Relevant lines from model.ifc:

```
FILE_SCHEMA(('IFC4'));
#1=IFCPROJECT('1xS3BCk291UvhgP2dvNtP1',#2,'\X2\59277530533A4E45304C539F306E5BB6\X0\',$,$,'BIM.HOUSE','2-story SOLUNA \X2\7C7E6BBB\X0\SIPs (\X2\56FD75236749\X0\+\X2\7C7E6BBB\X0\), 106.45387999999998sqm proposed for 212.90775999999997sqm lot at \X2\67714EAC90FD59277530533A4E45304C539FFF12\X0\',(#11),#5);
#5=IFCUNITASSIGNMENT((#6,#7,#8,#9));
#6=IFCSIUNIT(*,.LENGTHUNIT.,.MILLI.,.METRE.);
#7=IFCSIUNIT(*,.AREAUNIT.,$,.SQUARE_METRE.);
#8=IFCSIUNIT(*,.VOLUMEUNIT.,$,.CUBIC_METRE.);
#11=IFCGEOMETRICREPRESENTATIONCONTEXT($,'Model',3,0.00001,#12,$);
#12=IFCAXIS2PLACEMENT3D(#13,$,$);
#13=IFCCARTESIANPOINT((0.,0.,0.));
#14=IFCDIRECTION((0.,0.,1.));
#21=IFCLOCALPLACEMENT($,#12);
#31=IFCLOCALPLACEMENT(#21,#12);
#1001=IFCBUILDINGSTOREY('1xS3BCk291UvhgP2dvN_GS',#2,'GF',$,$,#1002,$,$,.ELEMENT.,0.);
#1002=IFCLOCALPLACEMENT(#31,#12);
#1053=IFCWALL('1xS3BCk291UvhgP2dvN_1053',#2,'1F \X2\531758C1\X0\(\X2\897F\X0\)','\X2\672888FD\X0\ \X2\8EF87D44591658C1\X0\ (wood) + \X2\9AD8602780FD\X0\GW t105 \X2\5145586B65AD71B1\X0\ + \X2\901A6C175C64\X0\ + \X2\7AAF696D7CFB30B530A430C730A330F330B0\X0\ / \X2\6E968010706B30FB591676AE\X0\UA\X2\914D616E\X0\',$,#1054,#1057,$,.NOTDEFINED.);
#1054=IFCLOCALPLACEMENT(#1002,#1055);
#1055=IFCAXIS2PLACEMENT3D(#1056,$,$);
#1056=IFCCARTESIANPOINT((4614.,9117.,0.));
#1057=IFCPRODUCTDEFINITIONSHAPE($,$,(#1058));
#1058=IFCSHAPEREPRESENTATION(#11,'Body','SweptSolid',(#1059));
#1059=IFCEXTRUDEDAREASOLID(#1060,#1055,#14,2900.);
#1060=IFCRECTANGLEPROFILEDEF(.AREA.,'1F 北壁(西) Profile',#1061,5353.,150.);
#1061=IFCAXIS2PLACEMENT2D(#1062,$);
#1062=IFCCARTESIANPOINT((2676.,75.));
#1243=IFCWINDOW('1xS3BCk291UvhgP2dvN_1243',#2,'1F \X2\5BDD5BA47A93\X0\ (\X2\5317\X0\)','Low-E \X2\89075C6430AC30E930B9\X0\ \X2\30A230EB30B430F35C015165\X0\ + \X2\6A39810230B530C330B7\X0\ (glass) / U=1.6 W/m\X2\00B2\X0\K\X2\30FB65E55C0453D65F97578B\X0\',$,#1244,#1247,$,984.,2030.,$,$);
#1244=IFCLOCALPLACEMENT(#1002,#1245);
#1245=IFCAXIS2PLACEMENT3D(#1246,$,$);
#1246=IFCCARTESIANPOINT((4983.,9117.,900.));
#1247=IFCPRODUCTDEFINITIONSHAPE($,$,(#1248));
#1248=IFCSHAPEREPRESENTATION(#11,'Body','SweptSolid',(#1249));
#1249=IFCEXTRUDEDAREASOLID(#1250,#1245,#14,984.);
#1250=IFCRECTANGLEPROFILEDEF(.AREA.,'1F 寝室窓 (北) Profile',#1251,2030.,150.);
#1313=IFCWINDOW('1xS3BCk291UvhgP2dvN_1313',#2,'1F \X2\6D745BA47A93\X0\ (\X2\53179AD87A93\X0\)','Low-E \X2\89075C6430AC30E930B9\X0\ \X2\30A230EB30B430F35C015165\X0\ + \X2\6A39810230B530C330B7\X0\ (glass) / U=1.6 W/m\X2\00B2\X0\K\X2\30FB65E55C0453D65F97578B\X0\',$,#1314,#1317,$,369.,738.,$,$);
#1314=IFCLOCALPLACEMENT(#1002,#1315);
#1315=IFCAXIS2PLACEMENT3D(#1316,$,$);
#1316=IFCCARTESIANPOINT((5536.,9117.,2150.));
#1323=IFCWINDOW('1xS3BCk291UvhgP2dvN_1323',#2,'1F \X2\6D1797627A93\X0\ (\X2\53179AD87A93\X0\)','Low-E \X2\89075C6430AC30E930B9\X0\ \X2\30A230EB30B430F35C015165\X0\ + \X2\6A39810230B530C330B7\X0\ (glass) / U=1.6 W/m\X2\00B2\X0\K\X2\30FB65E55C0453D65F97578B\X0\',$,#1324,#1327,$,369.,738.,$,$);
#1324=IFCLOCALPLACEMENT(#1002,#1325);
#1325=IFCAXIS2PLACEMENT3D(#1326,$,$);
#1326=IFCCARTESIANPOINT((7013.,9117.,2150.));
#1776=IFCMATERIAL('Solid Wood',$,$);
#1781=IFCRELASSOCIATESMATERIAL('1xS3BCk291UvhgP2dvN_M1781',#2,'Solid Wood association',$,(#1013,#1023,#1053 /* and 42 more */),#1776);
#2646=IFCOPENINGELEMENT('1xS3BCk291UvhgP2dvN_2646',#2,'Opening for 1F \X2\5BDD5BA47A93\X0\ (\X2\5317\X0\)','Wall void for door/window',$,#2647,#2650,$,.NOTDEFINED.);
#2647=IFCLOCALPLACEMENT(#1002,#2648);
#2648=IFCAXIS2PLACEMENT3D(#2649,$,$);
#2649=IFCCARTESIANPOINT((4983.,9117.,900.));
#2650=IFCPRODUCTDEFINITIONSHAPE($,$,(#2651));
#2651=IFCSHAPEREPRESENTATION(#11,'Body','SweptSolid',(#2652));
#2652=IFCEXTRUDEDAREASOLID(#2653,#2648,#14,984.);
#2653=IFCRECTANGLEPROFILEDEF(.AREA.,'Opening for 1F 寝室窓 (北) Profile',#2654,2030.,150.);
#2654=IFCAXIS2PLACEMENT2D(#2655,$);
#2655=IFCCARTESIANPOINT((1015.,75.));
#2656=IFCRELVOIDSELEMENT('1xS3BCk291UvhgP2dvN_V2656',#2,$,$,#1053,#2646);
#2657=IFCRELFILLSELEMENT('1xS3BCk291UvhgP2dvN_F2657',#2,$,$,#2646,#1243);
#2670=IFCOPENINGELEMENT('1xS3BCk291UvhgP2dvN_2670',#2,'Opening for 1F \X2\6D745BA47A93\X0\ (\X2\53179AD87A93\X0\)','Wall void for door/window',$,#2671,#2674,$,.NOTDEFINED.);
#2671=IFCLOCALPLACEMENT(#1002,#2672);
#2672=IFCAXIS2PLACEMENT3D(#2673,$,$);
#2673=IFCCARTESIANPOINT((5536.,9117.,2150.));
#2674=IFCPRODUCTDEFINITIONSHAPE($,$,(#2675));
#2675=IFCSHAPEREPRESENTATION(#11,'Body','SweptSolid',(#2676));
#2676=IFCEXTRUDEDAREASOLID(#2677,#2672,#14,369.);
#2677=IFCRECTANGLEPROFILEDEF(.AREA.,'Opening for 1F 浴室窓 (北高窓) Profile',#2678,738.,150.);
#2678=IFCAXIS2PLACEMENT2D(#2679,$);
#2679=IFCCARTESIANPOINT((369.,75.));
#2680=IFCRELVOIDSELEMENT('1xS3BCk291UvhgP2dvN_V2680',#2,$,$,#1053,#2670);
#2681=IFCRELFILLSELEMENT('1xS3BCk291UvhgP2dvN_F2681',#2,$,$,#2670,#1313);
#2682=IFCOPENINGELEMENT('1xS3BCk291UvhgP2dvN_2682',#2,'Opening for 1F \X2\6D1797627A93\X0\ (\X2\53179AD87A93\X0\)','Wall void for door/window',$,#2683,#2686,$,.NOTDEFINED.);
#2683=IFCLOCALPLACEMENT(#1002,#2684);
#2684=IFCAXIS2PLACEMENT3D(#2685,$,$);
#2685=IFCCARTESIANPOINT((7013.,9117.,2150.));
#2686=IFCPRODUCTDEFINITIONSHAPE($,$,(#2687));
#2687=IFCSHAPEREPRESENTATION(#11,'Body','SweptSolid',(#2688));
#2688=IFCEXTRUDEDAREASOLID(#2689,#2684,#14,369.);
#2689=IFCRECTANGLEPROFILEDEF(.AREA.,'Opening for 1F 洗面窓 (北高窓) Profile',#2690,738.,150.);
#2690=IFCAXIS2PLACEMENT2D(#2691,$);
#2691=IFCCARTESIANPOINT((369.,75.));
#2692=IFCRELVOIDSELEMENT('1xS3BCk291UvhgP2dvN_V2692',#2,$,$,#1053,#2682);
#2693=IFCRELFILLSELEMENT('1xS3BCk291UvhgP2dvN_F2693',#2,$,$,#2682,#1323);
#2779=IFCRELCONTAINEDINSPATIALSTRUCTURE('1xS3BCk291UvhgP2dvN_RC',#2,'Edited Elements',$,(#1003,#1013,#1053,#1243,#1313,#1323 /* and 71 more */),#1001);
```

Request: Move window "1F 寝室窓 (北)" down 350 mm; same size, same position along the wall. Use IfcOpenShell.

```python
import numpy as np
import ifcopenshell
import ifcopenshell.api.geometry
import ifcopenshell.util.placement
import ifcopenshell.util.unit

model = ifcopenshell.open("model.ifc")
unit_scale = ifcopenshell.util.unit.calculate_unit_scale(model)

window = model.by_guid("1xS3BCk291UvhgP2dvN_1243")
opening = window.FillsVoids[0].RelatingOpeningElement
dz = -0.35 / unit_scale

shift = np.array([0.0, 0.0, dz])
# The window is not placed relative to its opening, so move both.
for product in (opening, window):
    matrix = ifcopenshell.util.placement.get_local_placement(product.ObjectPlacement)
    matrix[:3, 3] += shift
    ifcopenshell.api.geometry.edit_object_placement(model, product=product, matrix=matrix, is_si=False)

print(f"moved by {dz * unit_scale:+.3f} m")

model.write("model_rev.ifc")
```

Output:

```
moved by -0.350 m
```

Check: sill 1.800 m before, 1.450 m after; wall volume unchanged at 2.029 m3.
